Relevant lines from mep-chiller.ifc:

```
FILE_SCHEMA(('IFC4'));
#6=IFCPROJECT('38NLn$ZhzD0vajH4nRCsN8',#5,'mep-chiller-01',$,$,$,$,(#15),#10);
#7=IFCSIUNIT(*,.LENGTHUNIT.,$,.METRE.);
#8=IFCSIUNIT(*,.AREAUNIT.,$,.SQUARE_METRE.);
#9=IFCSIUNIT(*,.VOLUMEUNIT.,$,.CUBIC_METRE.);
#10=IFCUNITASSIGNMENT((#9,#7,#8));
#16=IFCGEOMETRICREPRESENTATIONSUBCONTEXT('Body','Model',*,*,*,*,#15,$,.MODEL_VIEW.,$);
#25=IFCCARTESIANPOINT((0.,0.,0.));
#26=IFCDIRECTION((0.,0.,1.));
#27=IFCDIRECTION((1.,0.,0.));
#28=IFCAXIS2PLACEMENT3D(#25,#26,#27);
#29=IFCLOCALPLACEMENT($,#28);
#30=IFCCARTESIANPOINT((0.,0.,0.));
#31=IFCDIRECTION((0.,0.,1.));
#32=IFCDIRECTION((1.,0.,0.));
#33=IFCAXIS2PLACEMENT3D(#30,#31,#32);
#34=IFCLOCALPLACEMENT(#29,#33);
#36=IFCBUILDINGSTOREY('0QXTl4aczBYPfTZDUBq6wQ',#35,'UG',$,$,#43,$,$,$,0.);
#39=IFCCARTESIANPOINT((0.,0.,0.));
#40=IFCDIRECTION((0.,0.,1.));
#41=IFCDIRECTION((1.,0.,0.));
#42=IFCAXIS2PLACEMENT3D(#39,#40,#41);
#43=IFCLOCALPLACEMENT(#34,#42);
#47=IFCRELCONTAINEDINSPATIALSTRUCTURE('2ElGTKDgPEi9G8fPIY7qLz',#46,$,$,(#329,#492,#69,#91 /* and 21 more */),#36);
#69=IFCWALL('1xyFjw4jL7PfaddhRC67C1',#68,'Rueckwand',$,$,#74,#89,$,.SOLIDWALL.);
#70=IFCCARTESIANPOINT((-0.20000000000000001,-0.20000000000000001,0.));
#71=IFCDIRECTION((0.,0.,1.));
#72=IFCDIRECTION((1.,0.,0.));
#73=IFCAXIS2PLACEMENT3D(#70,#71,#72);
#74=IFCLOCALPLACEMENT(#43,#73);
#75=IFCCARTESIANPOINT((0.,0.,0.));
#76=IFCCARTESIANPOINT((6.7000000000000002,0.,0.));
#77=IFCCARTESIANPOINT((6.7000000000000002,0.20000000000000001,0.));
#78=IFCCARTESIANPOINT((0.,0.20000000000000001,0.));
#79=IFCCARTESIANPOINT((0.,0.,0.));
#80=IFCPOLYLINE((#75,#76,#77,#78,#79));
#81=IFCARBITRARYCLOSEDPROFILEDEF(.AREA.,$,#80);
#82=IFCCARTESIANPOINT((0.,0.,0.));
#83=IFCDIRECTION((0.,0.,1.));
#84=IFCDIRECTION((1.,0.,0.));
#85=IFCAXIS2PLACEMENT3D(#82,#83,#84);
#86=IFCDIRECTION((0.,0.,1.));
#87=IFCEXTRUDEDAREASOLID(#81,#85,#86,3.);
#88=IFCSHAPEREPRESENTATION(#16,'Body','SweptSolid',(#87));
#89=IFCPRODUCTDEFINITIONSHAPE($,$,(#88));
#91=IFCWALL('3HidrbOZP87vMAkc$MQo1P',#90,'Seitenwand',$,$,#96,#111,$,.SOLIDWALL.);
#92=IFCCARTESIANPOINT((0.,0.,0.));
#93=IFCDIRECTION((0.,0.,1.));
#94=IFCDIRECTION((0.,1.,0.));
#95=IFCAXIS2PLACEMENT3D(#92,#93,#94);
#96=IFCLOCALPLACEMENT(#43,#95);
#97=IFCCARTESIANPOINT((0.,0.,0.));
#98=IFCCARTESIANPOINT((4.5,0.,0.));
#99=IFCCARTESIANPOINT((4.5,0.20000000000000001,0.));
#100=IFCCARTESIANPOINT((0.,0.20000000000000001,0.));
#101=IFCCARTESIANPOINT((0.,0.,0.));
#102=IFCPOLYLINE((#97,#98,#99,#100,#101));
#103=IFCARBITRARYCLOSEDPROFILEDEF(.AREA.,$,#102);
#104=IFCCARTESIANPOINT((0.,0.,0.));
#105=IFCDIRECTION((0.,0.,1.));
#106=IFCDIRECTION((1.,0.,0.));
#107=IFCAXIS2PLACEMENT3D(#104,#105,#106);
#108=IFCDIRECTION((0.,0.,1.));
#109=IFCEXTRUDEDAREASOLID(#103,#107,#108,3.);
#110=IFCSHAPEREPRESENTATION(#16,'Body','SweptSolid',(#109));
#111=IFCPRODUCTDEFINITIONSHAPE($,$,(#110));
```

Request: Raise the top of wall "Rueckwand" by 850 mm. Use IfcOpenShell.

```python
import ifcopenshell
import ifcopenshell.geom
import ifcopenshell.util.representation
import ifcopenshell.util.shape
import ifcopenshell.util.unit

model = ifcopenshell.open("mep-chiller.ifc")
unit_scale = ifcopenshell.util.unit.calculate_unit_scale(model)
settings = ifcopenshell.geom.settings()


def volume(element):
    """Net volume in cubic metres, openings subtracted."""
    shape = ifcopenshell.geom.create_shape(settings, element)
    return ifcopenshell.util.shape.get_volume(shape.geometry)


wall = model.by_guid("1xyFjw4jL7PfaddhRC67C1")
before = volume(wall)

body = ifcopenshell.util.representation.get_representation(wall, "Model", "Body")
solid = body.Items[0]
old_height = solid.Depth
solid.Depth += 0.85 / unit_scale
after = volume(wall)

print(f"height {old_height:g} -> {solid.Depth:g}, volume {before:.3f} -> {after:.3f} m3")

model.write("mep-chiller_v2.ifc")
```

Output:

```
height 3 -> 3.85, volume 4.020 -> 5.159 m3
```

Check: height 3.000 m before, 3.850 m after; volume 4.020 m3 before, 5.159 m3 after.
